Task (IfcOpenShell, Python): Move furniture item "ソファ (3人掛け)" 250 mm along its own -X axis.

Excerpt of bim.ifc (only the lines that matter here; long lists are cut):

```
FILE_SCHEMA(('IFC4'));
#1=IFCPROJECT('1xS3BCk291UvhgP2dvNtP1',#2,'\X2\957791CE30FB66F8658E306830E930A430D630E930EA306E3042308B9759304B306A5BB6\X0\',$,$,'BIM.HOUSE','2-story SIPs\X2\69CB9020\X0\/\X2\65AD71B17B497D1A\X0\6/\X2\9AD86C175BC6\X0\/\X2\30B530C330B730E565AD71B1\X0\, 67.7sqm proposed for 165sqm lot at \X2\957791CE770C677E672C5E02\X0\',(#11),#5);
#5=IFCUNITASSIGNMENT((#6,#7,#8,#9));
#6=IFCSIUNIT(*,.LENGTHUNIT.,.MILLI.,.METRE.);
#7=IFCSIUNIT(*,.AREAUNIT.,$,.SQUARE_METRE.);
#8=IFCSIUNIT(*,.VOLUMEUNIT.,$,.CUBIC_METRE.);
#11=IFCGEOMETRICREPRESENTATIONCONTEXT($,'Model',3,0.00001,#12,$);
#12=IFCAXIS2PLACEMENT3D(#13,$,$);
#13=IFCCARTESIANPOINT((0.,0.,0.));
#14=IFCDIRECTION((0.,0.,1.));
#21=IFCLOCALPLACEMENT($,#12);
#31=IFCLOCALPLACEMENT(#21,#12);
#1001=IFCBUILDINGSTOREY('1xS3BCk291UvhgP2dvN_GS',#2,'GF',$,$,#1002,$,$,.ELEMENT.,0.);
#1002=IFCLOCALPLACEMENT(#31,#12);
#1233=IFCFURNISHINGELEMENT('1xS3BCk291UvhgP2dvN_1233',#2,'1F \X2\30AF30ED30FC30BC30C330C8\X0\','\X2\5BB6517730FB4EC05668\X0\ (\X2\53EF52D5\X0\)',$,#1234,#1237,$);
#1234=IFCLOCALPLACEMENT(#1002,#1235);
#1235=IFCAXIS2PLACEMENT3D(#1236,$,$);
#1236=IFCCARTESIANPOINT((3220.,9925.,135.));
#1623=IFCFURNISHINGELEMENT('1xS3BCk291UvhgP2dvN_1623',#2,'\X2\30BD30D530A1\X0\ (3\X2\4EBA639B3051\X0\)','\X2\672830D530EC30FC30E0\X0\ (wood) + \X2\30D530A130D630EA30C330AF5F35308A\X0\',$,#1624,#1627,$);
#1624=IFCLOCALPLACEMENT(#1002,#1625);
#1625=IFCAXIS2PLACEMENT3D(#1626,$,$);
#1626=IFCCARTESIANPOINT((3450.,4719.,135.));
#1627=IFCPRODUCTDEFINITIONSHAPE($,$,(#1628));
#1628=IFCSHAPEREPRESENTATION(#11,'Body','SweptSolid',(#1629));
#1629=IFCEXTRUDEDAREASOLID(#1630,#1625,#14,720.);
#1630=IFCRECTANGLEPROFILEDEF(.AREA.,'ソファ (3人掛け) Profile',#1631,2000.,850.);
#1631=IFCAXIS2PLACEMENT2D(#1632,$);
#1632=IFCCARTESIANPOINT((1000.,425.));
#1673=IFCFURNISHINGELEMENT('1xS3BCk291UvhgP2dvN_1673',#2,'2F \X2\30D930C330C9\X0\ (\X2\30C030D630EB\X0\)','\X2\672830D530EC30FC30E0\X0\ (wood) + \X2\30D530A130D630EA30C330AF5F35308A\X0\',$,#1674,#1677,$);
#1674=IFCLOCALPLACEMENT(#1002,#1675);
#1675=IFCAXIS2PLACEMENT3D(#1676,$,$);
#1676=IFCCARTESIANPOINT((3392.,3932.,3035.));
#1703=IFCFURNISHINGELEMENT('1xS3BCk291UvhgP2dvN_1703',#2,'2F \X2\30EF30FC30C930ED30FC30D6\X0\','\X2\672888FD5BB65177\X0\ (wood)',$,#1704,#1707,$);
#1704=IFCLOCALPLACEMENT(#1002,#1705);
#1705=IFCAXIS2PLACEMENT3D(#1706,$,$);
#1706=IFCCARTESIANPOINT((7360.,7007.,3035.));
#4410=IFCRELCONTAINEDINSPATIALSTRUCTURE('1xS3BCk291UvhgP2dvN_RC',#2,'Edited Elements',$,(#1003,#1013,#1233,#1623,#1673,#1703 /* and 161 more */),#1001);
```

```python
import ifcopenshell
import ifcopenshell.api.geometry
import ifcopenshell.util.placement
import ifcopenshell.util.unit

model = ifcopenshell.open("bim.ifc")
unit_scale = ifcopenshell.util.unit.calculate_unit_scale(model)

item = model.by_id(1623)
matrix = ifcopenshell.util.placement.get_local_placement(item.ObjectPlacement)
matrix[:3, 3] -= matrix[:3, 0] * 0.25 / unit_scale
ifcopenshell.api.geometry.edit_object_placement(model, product=item, matrix=matrix, is_si=False)

print(ifcopenshell.util.placement.get_local_placement(item.ObjectPlacement).round(3) + 0.0)

model.write("bim_updated.ifc")
```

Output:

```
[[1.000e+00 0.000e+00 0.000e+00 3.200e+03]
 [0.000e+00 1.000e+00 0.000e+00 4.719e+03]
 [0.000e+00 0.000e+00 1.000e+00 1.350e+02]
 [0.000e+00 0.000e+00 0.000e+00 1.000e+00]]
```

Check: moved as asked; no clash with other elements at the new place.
